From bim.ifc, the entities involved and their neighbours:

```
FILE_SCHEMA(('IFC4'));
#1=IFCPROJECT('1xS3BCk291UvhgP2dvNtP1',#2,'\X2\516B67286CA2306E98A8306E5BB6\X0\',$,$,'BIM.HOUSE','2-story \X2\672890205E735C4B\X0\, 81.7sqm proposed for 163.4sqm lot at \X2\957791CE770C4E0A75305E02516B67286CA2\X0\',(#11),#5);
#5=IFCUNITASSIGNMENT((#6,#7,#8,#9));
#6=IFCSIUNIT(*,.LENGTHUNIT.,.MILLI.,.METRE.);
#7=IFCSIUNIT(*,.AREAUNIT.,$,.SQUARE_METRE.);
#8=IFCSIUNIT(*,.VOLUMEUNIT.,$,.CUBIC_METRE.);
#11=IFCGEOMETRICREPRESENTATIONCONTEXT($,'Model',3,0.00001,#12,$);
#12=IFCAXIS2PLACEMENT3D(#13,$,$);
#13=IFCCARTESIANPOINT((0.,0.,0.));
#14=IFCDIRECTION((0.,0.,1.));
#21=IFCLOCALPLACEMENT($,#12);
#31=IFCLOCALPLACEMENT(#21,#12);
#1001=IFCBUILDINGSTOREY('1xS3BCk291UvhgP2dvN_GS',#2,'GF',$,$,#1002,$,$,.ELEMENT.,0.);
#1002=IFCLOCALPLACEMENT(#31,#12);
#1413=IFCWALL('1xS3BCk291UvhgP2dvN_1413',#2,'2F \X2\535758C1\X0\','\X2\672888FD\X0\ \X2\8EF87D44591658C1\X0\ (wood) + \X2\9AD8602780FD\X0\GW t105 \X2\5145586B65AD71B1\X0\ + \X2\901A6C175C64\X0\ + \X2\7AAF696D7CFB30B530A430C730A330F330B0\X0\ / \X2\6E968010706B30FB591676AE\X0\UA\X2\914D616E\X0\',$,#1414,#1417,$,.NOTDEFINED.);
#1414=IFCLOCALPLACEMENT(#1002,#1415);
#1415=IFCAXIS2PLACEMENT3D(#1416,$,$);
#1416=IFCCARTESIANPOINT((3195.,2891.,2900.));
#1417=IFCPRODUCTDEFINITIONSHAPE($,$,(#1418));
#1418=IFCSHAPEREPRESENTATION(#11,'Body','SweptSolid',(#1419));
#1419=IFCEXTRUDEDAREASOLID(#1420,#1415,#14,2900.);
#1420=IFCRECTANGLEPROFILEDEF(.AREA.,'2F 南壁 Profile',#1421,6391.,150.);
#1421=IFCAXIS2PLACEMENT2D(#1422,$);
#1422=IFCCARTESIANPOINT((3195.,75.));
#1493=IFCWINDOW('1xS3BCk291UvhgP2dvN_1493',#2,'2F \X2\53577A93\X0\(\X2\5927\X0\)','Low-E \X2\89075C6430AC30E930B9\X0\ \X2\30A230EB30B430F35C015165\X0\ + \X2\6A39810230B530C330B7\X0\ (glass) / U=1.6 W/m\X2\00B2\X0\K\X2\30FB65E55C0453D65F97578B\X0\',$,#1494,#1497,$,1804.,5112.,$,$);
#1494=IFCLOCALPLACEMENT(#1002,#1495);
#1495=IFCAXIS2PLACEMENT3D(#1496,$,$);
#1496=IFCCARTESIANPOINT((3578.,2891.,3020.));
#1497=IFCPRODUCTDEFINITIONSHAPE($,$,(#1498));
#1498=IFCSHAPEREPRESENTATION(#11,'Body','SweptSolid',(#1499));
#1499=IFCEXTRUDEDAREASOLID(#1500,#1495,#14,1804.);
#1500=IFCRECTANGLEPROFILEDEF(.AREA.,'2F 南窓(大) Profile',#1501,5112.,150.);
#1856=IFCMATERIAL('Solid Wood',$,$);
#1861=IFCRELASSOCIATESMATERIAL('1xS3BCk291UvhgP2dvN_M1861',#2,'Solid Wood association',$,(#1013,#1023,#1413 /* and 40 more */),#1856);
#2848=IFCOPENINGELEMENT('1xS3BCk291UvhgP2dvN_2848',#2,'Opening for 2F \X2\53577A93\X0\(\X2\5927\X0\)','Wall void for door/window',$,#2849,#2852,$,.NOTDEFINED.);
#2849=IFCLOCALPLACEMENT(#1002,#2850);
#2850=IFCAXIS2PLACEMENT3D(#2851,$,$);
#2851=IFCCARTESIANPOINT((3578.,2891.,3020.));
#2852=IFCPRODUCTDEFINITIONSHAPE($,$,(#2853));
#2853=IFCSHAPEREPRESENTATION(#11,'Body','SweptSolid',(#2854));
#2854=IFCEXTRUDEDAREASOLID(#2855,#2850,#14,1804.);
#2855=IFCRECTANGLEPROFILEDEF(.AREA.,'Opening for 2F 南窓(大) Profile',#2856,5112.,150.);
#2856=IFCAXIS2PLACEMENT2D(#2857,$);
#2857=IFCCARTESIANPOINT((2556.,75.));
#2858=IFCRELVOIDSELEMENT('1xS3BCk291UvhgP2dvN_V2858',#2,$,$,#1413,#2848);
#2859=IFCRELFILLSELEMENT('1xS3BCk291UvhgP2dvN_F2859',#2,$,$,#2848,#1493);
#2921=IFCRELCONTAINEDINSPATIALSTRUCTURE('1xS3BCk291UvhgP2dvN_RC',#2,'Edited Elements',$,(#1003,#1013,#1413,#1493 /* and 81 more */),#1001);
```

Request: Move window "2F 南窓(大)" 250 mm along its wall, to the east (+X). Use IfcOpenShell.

```python
import ifcopenshell
import ifcopenshell.api.geometry
import ifcopenshell.util.placement
import ifcopenshell.util.unit

model = ifcopenshell.open("bim.ifc")
unit_scale = ifcopenshell.util.unit.calculate_unit_scale(model)

window = model.by_guid("1xS3BCk291UvhgP2dvN_1493")
opening = window.FillsVoids[0].RelatingOpeningElement
wall = opening.VoidsElements[0].RelatingBuildingElement

wall_matrix = ifcopenshell.util.placement.get_local_placement(wall.ObjectPlacement)
shift = wall_matrix[:3, 0] * 0.25 / unit_scale
before = ifcopenshell.util.placement.get_local_placement(window.ObjectPlacement)[:3, 3].copy()

# The window is not placed relative to its opening, so move both.
for product in (opening, window):
    matrix = ifcopenshell.util.placement.get_local_placement(product.ObjectPlacement)
    matrix[:3, 3] += shift
    ifcopenshell.api.geometry.edit_object_placement(model, product=product, matrix=matrix, is_si=False)

after = ifcopenshell.util.placement.get_local_placement(window.ObjectPlacement)[:3, 3]
print("window moved by", (after - before).round(3) + 0.0)

model.write("bim_rev.ifc")
```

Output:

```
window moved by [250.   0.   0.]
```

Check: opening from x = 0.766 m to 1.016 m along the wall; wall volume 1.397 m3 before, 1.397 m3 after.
